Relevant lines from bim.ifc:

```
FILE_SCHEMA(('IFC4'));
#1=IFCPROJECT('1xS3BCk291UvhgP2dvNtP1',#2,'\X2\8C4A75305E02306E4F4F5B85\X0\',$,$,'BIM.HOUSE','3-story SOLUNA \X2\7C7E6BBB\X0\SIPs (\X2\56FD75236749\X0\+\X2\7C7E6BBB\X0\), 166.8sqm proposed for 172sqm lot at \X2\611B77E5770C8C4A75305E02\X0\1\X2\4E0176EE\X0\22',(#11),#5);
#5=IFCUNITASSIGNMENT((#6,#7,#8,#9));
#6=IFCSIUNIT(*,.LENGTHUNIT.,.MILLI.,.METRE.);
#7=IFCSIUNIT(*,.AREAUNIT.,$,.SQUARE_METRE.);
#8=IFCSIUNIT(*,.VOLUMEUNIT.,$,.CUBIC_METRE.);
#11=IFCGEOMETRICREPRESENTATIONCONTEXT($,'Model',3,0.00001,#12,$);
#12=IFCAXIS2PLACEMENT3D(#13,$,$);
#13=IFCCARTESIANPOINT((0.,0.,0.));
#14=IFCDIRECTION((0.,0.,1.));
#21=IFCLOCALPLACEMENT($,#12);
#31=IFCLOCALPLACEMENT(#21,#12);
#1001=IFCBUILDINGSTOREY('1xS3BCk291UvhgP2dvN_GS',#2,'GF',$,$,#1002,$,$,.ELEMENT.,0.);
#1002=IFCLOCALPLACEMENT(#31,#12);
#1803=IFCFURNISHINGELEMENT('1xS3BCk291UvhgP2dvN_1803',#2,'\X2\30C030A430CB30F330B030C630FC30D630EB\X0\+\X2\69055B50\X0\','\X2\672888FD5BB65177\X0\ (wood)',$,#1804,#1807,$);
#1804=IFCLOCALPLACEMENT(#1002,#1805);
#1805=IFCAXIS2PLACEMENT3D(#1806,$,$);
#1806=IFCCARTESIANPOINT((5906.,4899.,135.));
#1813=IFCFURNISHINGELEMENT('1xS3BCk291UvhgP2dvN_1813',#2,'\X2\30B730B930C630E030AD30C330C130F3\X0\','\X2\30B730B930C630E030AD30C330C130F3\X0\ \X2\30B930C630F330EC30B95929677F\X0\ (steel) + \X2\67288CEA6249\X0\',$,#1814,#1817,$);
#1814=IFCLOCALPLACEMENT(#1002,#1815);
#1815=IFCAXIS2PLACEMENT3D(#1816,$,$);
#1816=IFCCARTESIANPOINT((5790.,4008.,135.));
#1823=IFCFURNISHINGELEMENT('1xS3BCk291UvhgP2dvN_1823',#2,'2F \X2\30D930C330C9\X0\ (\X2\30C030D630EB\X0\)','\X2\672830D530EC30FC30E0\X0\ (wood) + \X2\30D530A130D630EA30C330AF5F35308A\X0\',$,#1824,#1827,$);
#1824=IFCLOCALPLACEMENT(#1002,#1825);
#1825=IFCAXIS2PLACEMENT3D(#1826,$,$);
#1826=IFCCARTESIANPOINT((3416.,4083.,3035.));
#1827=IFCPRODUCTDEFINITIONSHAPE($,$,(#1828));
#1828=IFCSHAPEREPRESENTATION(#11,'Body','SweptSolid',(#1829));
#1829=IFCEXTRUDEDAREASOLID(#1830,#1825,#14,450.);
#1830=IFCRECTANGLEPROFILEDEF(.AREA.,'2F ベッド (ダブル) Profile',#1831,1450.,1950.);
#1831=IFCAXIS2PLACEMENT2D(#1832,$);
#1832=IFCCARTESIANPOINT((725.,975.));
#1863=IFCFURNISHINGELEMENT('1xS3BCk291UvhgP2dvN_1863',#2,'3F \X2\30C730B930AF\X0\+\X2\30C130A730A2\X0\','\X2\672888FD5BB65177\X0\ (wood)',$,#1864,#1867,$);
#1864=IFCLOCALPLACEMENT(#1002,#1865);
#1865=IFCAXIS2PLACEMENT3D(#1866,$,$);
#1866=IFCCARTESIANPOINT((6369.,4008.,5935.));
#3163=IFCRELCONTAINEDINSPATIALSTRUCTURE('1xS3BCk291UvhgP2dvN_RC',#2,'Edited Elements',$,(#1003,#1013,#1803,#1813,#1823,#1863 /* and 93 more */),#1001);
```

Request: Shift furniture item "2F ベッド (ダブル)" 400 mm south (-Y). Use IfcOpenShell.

```python
import ifcopenshell
import ifcopenshell.api.geometry
import ifcopenshell.util.placement
import ifcopenshell.util.unit

model = ifcopenshell.open("bim.ifc")
unit_scale = ifcopenshell.util.unit.calculate_unit_scale(model)

item = model.by_guid("1xS3BCk291UvhgP2dvN_1823")
matrix = ifcopenshell.util.placement.get_local_placement(item.ObjectPlacement)
matrix[1, 3] -= 0.4 / unit_scale
ifcopenshell.api.geometry.edit_object_placement(model, product=item, matrix=matrix, is_si=False)

print(ifcopenshell.util.placement.get_local_placement(item.ObjectPlacement).round(3) + 0.0)

model.write("bim_updated.ifc")
```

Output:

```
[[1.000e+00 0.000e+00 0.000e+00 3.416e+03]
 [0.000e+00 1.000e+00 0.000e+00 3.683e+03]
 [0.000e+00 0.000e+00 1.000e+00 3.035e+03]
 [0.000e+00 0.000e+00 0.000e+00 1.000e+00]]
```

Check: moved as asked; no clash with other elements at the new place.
